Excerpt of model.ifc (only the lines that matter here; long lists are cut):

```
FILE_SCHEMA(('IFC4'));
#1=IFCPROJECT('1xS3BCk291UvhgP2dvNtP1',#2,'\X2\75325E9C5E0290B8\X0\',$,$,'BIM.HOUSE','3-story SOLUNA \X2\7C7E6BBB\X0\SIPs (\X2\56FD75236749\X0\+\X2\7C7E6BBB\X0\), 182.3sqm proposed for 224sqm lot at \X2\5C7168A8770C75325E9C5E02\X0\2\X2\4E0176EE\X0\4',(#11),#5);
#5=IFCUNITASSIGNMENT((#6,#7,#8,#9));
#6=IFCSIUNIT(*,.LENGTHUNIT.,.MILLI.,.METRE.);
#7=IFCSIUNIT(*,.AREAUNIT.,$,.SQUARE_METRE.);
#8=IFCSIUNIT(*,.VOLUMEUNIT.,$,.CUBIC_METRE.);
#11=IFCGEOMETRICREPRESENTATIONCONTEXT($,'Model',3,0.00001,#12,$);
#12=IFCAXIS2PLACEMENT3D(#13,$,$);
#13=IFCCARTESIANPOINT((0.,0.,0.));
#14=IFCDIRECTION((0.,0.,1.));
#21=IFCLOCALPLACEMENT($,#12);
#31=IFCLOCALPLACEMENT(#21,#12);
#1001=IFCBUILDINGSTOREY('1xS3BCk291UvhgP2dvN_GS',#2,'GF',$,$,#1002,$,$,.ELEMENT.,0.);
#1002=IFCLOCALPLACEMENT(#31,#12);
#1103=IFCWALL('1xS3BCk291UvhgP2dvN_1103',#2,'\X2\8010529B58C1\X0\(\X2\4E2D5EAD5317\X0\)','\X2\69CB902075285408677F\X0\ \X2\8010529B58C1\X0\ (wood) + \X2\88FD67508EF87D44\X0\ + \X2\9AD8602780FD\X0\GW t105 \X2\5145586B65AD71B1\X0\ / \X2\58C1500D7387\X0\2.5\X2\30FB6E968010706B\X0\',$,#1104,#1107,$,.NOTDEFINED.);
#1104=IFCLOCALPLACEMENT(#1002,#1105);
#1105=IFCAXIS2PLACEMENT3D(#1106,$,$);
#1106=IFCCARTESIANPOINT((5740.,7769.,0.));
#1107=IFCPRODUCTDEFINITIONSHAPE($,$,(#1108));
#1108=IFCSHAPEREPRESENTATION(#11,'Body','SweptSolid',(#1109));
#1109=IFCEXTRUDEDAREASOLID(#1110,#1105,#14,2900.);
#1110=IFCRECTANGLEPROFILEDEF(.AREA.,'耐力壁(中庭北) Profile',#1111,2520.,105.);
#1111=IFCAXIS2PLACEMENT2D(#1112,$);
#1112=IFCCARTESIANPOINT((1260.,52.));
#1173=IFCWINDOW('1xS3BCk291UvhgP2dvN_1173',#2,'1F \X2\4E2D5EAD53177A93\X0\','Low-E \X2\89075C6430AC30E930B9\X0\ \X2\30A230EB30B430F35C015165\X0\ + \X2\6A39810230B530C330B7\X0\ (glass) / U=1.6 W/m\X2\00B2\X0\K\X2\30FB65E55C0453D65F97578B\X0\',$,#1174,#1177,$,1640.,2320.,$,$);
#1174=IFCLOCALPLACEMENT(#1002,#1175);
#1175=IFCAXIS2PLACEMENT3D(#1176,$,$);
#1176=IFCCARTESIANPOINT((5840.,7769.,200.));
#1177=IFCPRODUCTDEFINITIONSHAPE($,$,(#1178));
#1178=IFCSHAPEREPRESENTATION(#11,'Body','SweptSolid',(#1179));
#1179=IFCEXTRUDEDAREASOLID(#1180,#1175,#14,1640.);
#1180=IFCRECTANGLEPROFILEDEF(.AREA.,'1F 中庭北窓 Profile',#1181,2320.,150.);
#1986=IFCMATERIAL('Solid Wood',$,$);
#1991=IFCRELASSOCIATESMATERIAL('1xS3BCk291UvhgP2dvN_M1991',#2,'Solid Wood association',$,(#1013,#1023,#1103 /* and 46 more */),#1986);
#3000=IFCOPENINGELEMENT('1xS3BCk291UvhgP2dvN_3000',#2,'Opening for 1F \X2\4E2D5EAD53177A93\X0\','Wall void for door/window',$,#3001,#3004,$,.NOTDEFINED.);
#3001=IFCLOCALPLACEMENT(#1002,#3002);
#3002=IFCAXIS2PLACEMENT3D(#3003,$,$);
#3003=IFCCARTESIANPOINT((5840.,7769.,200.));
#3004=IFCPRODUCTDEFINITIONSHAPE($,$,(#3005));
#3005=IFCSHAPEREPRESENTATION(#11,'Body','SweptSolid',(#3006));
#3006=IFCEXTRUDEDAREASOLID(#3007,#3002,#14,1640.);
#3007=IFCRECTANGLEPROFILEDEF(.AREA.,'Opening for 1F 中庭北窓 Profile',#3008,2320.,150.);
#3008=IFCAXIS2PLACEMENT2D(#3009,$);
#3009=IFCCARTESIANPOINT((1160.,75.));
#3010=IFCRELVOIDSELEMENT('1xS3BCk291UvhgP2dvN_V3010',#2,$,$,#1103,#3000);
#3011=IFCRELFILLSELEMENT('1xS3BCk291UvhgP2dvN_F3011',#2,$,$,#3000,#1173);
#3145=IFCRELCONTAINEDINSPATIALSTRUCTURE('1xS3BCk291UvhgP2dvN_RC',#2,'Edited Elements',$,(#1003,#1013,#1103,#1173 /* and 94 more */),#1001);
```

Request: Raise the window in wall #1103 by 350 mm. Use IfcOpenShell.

```python
import numpy as np
import ifcopenshell
import ifcopenshell.api.geometry
import ifcopenshell.util.placement
import ifcopenshell.util.unit

model = ifcopenshell.open("model.ifc")
unit_scale = ifcopenshell.util.unit.calculate_unit_scale(model)

window = model.by_guid("1xS3BCk291UvhgP2dvN_1173")
opening = window.FillsVoids[0].RelatingOpeningElement
dz = 350.0

shift = np.array([0.0, 0.0, dz])
# The window is not placed relative to its opening, so move both.
for product in (opening, window):
    matrix = ifcopenshell.util.placement.get_local_placement(product.ObjectPlacement)
    matrix[:3, 3] += shift
    ifcopenshell.api.geometry.edit_object_placement(model, product=product, matrix=matrix, is_si=False)

print(f"moved by {dz * unit_scale:+.3f} m")

model.write("model_updated.ifc")
```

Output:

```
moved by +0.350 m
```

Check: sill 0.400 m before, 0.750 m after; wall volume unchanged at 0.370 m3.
